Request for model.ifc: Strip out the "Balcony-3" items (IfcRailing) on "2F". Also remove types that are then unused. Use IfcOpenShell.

First a look at what the model holds.

```python
import ifcopenshell
import ifcopenshell.util.element

model = ifcopenshell.open("model.ifc")
print(model.schema)
storey = next(s for s in model.by_type("IfcBuildingStorey") if s.Name == "2F")
railings = [e for e in ifcopenshell.util.element.get_decomposition(storey) if e.is_a("IfcRailing")]
seen = {}
for e in railings:
    element_type = ifcopenshell.util.element.get_type(e)
    name = element_type.Name if element_type not in (None, e) else None
    seen[name] = seen.get(name, 0) + 1
for name, count in sorted(seen.items(), key=str):
    print(count, "x", name)
```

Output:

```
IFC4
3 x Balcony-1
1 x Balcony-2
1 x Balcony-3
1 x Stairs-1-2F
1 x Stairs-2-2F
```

```python
import ifcopenshell
import ifcopenshell.api.root
import ifcopenshell.util.element

model = ifcopenshell.open("model.ifc")

storey = next(s for s in model.by_type("IfcBuildingStorey") if s.Name == "2F")
railings = [e for e in ifcopenshell.util.element.get_decomposition(storey) if e.is_a("IfcRailing")]
targets = [e for e in railings if (t := ifcopenshell.util.element.get_type(e)) not in (None, e) and t.Name == "Balcony-3"]
types = {ifcopenshell.util.element.get_type(e) for e in targets} - {None, *targets}

for e in targets:
    ifcopenshell.api.root.remove_product(model, product=e)
print(len(targets), "removed")

unused = [t for t in types if not ifcopenshell.util.element.get_types(t)]
for t in unused:
    ifcopenshell.api.root.remove_product(model, product=t)
print(len(unused), "unused types removed")

model.write("model_edited.ifc")
```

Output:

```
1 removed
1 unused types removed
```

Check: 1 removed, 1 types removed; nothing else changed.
